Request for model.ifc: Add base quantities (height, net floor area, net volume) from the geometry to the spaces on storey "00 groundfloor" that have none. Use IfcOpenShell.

First a look at what the model holds.

```python
import ifcopenshell
import ifcopenshell.util.element
import ifcopenshell.util.unit

model = ifcopenshell.open("model.ifc")
print(model.schema)
for unit_type in ("LENGTHUNIT", "AREAUNIT", "VOLUMEUNIT"):
    print(unit_type, ifcopenshell.util.unit.calculate_unit_scale(model, unit_type))
storey = next(s for s in model.by_type("IfcBuildingStorey") if s.Name == "00 groundfloor")
spaces = [e for e in ifcopenshell.util.element.get_decomposition(storey) if e.is_a("IfcSpace")]
for e in sorted(spaces, key=lambda e: e.id()):
    print(e.id(), e.is_a(), e.Name, list(ifcopenshell.util.element.get_psets(e, qtos_only=True)), sep=" | ")
```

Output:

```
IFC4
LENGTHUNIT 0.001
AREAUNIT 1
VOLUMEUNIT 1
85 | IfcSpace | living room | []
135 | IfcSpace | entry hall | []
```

```python
import ifcopenshell
import ifcopenshell.api.pset
import ifcopenshell.geom
import ifcopenshell.util.element
import ifcopenshell.util.shape
import ifcopenshell.util.unit

model = ifcopenshell.open("model.ifc")
unit_scale = ifcopenshell.util.unit.calculate_unit_scale(model)
area_scale = ifcopenshell.util.unit.calculate_unit_scale(model, "AREAUNIT")
volume_scale = ifcopenshell.util.unit.calculate_unit_scale(model, "VOLUMEUNIT")
settings = ifcopenshell.geom.settings()

storey = next(s for s in model.by_type("IfcBuildingStorey") if s.Name == "00 groundfloor")
spaces = [e for e in ifcopenshell.util.element.get_decomposition(storey) if e.is_a("IfcSpace")]

for e in sorted(spaces, key=lambda e: e.id()):
    if ifcopenshell.util.element.get_psets(e, qtos_only=True, should_inherit=False):
        continue
    # Geometry comes back in metres, in the element's own axes.
    shape = ifcopenshell.geom.create_shape(settings, e)
    values = {
        "Height": ifcopenshell.util.shape.get_z(shape.geometry) / unit_scale,
        "NetFloorArea": ifcopenshell.util.shape.get_footprint_area(shape.geometry) / area_scale,
        "NetVolume": ifcopenshell.util.shape.get_volume(shape.geometry) / volume_scale,
    }
    qto = ifcopenshell.api.pset.add_qto(model, product=e, name="Qto_SpaceBaseQuantities")
    ifcopenshell.api.pset.edit_qto(model, qto=qto, properties=values)
    print(e.id(), {k: round(v, 3) for k, v in values.items()})

model.write("model_v2.ifc")
```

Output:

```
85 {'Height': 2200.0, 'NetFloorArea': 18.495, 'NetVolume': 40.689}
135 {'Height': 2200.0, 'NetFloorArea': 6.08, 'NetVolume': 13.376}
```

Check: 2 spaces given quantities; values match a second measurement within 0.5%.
